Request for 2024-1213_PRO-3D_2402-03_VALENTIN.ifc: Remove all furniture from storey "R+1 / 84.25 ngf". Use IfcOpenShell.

First a look at what the model holds.

```python
import ifcopenshell
import ifcopenshell.util.element

model = ifcopenshell.open("2024-1213_PRO-3D_2402-03_VALENTIN.ifc")
print(model.schema)
storey = next(s for s in model.by_type("IfcBuildingStorey") if s.Name == "R+1 / 84.25 ngf")
furniture = [e for e in ifcopenshell.util.element.get_decomposition(storey) if e.is_a("IfcFurnishingElement")]
seen = {}
for e in furniture:
    element_type = ifcopenshell.util.element.get_type(e)
    name = element_type.Name if element_type not in (None, e) else None
    seen[name] = seen.get(name, 0) + 1
for name, count in sorted(seen.items(), key=str):
    print(count, "x", name)
```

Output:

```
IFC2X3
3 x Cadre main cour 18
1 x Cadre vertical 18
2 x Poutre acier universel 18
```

```python
import ifcopenshell
import ifcopenshell.api.root
import ifcopenshell.util.element

model = ifcopenshell.open("2024-1213_PRO-3D_2402-03_VALENTIN.ifc")

storey = next(s for s in model.by_type("IfcBuildingStorey") if s.Name == "R+1 / 84.25 ngf")
furniture = [e for e in ifcopenshell.util.element.get_decomposition(storey) if e.is_a("IfcFurnishingElement")]

for e in furniture:
    ifcopenshell.api.root.remove_product(model, product=e)
print(len(furniture), "removed")

model.write("2024-1213_PRO-3D_2402-03_VALENTIN_updated.ifc")
```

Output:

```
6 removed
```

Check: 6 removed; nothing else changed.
